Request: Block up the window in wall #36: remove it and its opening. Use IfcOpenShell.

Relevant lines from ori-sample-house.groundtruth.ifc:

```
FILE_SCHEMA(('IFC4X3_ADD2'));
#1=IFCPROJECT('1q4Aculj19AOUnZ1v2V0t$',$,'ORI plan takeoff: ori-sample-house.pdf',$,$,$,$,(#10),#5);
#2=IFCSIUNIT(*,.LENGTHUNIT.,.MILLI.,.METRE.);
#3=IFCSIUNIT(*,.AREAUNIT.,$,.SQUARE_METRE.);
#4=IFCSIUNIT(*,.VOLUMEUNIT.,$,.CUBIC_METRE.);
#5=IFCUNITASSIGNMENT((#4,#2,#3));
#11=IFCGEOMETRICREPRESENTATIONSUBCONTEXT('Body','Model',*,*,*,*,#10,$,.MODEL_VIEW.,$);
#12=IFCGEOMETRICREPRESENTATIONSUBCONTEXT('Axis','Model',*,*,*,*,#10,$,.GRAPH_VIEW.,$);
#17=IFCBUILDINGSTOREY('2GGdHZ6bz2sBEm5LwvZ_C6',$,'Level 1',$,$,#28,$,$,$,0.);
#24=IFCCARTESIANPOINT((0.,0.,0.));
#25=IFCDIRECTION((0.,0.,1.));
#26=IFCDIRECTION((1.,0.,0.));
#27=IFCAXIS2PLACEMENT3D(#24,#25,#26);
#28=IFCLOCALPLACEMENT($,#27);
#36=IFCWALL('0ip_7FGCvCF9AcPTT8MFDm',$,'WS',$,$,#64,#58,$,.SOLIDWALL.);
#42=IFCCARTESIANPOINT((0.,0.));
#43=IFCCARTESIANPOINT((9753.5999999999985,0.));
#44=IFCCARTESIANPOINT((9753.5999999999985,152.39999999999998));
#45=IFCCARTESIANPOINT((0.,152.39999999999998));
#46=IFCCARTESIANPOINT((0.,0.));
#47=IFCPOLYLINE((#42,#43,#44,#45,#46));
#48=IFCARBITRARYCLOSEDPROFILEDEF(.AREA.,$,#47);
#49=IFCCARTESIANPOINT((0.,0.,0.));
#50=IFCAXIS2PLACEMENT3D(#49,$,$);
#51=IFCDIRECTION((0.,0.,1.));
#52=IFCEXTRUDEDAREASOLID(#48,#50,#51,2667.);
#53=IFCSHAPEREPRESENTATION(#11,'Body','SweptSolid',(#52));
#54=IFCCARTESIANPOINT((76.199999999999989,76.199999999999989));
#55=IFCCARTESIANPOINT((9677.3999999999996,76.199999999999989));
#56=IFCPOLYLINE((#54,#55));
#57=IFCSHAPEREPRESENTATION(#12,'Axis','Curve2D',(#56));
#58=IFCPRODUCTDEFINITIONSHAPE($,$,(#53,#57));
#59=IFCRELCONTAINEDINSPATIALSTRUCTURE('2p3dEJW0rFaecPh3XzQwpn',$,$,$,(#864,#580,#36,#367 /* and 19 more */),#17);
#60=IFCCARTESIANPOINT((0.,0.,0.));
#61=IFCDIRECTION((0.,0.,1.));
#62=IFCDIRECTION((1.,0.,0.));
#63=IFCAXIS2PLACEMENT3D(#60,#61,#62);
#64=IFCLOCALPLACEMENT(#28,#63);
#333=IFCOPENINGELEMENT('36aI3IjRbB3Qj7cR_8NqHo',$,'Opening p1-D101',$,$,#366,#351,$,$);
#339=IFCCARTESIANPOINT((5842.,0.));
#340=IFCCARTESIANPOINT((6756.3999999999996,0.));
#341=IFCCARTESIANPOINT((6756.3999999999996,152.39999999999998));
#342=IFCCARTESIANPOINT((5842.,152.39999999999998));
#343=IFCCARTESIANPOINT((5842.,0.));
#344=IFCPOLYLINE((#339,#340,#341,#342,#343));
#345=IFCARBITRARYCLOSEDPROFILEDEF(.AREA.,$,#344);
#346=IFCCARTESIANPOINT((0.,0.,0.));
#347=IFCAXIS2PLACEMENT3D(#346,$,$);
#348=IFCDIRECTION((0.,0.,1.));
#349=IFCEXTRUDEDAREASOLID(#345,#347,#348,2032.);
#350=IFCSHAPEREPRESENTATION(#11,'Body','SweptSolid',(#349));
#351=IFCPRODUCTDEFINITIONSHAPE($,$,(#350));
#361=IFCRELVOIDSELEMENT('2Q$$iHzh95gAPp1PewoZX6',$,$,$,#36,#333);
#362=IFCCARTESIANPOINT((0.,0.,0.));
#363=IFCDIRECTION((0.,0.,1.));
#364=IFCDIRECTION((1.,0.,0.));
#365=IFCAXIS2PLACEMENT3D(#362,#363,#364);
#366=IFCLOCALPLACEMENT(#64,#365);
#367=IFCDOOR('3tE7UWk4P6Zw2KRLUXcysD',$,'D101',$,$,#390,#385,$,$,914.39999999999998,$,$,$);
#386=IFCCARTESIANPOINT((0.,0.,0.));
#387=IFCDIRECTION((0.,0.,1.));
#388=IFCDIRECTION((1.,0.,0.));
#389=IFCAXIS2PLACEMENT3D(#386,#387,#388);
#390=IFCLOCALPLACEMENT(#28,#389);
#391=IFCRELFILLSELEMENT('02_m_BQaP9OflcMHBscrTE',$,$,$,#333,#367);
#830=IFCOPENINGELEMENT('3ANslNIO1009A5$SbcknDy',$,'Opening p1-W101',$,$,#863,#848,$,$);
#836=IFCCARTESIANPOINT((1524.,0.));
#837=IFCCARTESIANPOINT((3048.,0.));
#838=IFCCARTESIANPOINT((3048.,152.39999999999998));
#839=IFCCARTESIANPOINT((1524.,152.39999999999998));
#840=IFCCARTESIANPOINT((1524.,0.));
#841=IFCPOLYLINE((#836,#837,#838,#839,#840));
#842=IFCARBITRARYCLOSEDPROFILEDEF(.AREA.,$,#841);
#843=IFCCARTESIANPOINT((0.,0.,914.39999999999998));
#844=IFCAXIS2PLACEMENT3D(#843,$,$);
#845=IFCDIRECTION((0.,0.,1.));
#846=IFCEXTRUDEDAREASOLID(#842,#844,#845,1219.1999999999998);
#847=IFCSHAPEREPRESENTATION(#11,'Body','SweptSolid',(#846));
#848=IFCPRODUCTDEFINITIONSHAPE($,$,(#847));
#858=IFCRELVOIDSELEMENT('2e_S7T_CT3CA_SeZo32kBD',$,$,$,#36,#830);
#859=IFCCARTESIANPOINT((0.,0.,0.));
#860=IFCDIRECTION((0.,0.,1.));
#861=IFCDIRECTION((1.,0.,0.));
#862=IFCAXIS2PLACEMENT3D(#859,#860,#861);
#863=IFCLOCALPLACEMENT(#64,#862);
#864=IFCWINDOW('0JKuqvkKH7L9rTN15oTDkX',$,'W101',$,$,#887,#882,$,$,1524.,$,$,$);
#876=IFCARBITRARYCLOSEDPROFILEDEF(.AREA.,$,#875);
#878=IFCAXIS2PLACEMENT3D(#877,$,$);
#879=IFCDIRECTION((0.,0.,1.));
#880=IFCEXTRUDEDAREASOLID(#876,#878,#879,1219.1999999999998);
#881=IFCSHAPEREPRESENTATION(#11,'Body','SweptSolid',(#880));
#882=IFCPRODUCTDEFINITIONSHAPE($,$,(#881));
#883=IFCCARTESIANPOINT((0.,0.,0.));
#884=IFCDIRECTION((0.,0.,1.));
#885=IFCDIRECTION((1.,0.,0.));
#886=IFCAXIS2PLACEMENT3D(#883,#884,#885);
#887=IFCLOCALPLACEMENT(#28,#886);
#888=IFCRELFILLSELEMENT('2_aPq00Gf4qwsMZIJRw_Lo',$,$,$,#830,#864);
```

```python
import ifcopenshell
import ifcopenshell.api.feature
import ifcopenshell.api.root
import ifcopenshell.geom
import ifcopenshell.util.shape

model = ifcopenshell.open("ori-sample-house.groundtruth.ifc")
settings = ifcopenshell.geom.settings()


def volume(element):
    """Net volume in cubic metres, openings subtracted."""
    shape = ifcopenshell.geom.create_shape(settings, element)
    return ifcopenshell.util.shape.get_volume(shape.geometry)


window = model.by_guid("0JKuqvkKH7L9rTN15oTDkX")
opening = window.FillsVoids[0].RelatingOpeningElement
wall = opening.VoidsElements[0].RelatingBuildingElement
before = volume(wall)

ifcopenshell.api.root.remove_product(model, product=window)
ifcopenshell.api.feature.remove_feature(model, feature=opening)

after = volume(wall)

print(f"wall volume {before:.3f} -> {after:.3f} m3")

model.write("ori-sample-house.groundtruth-out.ifc")
```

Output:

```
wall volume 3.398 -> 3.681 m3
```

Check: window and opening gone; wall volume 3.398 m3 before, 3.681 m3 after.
